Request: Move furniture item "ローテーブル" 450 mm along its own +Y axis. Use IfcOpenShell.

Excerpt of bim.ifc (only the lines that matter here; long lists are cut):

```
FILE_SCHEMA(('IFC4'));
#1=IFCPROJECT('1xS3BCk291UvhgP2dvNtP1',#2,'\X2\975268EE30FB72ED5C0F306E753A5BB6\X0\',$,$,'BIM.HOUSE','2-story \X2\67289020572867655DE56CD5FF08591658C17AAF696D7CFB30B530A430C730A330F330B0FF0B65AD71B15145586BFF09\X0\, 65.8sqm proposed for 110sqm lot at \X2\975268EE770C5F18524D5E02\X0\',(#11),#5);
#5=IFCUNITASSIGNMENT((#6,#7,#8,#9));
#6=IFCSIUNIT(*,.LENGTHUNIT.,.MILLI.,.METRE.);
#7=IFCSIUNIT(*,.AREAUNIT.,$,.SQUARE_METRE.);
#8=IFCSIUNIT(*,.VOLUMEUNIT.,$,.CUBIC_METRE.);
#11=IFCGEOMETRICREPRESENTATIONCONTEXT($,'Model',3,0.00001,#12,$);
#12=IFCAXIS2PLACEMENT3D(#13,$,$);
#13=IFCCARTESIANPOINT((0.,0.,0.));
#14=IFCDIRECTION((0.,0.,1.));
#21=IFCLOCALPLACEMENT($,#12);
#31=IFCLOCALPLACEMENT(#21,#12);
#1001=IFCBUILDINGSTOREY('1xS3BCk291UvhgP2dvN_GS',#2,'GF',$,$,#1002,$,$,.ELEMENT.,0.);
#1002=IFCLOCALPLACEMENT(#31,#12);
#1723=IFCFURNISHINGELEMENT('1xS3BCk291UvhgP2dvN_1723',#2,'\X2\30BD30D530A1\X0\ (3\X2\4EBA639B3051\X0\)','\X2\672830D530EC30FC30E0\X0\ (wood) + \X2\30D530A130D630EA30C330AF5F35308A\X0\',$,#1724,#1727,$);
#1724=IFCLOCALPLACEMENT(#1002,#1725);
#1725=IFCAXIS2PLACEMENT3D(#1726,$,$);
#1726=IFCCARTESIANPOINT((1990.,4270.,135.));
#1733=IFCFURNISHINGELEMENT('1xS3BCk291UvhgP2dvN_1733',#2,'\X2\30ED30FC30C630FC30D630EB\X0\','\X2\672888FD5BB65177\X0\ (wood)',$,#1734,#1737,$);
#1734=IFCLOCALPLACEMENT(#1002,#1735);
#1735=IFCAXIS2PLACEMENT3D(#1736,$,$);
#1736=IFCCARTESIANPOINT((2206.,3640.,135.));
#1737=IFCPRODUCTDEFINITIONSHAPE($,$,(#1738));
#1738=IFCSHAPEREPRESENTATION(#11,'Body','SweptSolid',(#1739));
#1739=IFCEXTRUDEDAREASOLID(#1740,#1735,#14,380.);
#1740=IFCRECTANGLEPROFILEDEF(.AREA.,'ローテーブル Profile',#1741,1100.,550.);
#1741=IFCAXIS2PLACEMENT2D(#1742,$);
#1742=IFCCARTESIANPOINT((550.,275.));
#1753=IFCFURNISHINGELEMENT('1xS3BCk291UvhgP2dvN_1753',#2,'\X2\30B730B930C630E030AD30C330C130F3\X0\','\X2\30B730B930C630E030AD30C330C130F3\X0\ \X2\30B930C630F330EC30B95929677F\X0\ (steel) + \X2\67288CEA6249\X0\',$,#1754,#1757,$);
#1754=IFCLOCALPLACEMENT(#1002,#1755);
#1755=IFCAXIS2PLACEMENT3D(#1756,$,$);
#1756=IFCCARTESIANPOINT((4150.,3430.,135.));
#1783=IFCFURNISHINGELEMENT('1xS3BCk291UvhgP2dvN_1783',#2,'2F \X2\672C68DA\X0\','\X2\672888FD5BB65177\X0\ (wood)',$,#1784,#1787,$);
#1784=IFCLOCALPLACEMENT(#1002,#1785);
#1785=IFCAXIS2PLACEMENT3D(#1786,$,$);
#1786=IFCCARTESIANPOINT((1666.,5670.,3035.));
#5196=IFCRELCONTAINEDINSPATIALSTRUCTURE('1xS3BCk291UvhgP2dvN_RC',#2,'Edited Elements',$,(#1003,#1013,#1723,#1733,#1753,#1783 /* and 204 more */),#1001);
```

```python
import ifcopenshell
import ifcopenshell.api.geometry
import ifcopenshell.util.placement

model = ifcopenshell.open("bim.ifc")

item = model.by_guid("1xS3BCk291UvhgP2dvN_1733")
matrix = ifcopenshell.util.placement.get_local_placement(item.ObjectPlacement)
matrix[:3, 3] += matrix[:3, 1] * 450.0
ifcopenshell.api.geometry.edit_object_placement(model, product=item, matrix=matrix, is_si=False)

print(ifcopenshell.util.placement.get_local_placement(item.ObjectPlacement).round(3) + 0.0)

model.write("bim-out.ifc")
```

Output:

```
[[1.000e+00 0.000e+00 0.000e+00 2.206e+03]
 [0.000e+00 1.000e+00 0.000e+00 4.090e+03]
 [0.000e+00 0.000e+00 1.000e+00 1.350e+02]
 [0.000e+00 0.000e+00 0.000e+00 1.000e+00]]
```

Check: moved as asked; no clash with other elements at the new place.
